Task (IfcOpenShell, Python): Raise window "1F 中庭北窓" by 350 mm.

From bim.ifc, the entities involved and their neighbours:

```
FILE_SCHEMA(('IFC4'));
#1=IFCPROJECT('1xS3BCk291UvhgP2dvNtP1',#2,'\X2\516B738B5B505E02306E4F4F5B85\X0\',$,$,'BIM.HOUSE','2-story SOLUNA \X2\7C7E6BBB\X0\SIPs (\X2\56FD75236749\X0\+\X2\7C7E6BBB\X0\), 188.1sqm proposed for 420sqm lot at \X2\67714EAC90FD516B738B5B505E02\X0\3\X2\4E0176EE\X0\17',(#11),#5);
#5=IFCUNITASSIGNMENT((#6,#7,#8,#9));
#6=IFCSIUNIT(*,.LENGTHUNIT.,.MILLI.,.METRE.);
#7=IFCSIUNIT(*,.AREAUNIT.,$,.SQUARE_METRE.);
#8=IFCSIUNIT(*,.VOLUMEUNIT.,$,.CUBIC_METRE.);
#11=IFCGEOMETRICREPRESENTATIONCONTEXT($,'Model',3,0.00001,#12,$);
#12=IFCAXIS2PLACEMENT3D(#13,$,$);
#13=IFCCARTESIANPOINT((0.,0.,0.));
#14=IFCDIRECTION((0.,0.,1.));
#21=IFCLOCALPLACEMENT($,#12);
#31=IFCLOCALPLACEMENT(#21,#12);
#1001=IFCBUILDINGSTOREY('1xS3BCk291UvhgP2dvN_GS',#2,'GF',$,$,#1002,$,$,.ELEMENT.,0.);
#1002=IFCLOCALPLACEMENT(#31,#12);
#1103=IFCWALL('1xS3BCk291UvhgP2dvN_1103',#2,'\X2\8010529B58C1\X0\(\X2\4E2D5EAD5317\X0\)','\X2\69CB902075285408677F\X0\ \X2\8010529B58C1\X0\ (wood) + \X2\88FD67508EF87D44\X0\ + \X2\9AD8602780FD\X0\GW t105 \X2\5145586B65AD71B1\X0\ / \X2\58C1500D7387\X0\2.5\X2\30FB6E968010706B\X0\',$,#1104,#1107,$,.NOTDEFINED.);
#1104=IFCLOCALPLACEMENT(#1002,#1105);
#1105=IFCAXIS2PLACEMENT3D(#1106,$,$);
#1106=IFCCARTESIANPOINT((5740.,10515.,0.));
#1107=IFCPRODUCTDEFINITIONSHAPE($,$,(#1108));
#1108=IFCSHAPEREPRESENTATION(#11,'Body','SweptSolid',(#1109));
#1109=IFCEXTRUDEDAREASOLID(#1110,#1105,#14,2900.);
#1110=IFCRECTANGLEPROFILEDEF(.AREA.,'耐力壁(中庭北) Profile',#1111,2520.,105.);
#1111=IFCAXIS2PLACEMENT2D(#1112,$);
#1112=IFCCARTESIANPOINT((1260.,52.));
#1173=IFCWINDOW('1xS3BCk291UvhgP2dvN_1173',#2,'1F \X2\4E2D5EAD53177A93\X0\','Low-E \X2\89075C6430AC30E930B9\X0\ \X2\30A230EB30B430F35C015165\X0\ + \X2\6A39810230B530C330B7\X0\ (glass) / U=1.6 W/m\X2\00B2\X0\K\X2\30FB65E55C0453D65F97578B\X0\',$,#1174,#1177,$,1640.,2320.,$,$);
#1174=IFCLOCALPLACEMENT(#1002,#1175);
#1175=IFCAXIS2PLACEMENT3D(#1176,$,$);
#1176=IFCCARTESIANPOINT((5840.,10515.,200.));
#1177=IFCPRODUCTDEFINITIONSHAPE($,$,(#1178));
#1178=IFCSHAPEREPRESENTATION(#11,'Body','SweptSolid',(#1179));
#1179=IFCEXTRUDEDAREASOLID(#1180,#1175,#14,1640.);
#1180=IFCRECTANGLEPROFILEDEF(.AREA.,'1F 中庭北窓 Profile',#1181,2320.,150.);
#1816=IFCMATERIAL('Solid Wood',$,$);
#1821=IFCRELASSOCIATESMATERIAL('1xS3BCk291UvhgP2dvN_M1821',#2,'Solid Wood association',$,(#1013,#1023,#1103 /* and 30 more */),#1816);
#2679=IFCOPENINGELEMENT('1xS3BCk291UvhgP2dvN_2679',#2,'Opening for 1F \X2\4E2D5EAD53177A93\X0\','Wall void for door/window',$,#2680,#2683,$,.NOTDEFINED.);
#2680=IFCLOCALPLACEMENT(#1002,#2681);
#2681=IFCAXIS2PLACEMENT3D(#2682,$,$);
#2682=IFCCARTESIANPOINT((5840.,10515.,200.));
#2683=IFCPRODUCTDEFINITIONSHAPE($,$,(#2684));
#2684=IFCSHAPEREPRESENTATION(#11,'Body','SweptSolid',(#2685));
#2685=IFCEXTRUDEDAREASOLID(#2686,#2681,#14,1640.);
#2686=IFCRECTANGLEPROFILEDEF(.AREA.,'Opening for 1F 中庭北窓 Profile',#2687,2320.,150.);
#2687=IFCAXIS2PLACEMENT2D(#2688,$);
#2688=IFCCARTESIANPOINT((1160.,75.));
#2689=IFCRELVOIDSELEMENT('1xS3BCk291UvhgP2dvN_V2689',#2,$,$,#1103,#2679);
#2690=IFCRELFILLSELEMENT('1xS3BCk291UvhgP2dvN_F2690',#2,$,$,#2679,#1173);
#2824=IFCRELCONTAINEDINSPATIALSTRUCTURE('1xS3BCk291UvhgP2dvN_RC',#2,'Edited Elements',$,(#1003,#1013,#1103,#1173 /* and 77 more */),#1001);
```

```python
import numpy as np
import ifcopenshell
import ifcopenshell.api.geometry
import ifcopenshell.util.placement
import ifcopenshell.util.unit

model = ifcopenshell.open("bim.ifc")
unit_scale = ifcopenshell.util.unit.calculate_unit_scale(model)

window = model.by_id(1173)
opening = window.FillsVoids[0].RelatingOpeningElement
dz = 350.0

shift = np.array([0.0, 0.0, dz])
# The window is not placed relative to its opening, so move both.
for product in (opening, window):
    matrix = ifcopenshell.util.placement.get_local_placement(product.ObjectPlacement)
    matrix[:3, 3] += shift
    ifcopenshell.api.geometry.edit_object_placement(model, product=product, matrix=matrix, is_si=False)

print(f"moved by {dz * unit_scale:+.3f} m")

model.write("bim_updated.ifc")
```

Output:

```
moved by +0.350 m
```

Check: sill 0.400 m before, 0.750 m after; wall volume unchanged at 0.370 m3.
